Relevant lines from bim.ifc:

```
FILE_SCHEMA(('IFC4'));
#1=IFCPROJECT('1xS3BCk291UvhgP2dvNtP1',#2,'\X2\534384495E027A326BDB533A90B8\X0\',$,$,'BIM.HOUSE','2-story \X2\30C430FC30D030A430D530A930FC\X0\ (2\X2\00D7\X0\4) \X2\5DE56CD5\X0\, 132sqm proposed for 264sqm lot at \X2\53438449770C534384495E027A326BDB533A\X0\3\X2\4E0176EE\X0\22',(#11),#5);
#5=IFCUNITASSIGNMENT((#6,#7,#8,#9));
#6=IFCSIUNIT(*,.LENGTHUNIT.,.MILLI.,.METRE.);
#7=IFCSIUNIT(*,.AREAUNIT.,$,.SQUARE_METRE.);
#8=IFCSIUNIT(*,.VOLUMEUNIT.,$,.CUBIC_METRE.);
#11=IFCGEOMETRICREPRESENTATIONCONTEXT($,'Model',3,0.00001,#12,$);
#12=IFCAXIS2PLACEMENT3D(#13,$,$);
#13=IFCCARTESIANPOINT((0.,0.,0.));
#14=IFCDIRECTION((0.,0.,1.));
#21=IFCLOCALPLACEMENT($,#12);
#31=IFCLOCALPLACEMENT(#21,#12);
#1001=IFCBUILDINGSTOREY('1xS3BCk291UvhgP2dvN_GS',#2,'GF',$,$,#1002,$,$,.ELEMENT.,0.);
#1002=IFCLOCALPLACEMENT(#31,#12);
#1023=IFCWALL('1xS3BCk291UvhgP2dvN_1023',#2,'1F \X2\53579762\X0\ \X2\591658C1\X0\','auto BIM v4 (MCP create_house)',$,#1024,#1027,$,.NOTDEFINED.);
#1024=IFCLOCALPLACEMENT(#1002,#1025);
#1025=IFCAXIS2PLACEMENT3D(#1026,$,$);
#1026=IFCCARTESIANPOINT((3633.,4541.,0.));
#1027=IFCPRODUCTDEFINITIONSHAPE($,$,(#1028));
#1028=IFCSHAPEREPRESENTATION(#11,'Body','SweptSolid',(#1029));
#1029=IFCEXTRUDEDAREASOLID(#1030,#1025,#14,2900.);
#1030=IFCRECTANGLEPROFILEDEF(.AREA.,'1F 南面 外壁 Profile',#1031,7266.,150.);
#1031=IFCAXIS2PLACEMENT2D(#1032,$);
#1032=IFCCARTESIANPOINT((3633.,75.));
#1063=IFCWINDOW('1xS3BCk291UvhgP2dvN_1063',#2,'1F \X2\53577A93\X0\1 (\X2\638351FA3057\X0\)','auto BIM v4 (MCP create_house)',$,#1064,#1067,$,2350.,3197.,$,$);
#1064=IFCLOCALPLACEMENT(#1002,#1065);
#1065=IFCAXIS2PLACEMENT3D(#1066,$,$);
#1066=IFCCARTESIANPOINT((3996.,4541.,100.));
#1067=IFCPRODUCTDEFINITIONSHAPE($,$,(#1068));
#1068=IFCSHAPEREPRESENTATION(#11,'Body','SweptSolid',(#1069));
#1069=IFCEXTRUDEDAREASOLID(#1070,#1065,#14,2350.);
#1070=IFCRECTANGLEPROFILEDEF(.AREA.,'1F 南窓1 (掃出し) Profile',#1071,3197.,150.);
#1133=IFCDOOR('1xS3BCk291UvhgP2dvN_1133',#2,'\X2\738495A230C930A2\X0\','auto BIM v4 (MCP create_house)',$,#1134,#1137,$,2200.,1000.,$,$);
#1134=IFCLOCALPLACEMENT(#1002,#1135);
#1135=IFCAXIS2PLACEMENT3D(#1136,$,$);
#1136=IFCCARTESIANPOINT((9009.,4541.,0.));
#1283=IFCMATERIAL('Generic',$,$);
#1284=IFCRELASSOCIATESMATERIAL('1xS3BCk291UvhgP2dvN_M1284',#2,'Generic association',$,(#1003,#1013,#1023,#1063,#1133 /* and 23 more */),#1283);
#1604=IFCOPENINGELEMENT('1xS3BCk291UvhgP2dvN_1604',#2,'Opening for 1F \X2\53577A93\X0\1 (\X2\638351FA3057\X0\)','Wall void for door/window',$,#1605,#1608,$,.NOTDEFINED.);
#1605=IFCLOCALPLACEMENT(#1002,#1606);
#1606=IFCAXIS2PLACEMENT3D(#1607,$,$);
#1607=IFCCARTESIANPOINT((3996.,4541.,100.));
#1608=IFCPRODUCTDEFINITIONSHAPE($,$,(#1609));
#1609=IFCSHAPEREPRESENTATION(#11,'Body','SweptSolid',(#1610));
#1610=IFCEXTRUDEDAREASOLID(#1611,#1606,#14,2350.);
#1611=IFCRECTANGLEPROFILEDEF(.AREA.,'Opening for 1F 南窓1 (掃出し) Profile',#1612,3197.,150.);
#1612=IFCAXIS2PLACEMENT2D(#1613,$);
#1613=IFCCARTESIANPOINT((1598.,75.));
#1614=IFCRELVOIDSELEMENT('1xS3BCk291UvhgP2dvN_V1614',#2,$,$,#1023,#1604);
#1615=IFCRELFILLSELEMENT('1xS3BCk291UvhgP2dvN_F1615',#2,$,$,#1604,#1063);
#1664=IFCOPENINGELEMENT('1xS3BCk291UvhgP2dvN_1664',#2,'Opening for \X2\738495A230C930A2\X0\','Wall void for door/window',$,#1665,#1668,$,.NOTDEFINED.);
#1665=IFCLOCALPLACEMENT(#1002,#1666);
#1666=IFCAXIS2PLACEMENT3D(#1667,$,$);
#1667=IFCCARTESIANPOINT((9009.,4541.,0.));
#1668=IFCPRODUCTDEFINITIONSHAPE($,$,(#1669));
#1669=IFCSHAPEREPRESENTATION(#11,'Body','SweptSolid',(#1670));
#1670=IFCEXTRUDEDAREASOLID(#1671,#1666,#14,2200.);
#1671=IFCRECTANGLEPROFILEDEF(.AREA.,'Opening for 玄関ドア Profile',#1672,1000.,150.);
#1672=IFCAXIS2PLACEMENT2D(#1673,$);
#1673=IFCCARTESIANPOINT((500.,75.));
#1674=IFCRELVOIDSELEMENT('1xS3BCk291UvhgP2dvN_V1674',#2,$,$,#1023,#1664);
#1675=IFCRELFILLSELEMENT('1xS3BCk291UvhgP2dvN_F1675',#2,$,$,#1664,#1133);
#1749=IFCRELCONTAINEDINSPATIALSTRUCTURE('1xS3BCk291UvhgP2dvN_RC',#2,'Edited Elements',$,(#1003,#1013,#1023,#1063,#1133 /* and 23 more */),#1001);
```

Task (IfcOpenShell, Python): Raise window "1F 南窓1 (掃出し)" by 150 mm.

```python
import numpy as np
import ifcopenshell
import ifcopenshell.api.geometry
import ifcopenshell.util.placement
import ifcopenshell.util.unit

model = ifcopenshell.open("bim.ifc")
unit_scale = ifcopenshell.util.unit.calculate_unit_scale(model)

window = model.by_guid("1xS3BCk291UvhgP2dvN_1063")
opening = window.FillsVoids[0].RelatingOpeningElement
dz = 0.15 / unit_scale

shift = np.array([0.0, 0.0, dz])
# The window is not placed relative to its opening, so move both.
for product in (opening, window):
    matrix = ifcopenshell.util.placement.get_local_placement(product.ObjectPlacement)
    matrix[:3, 3] += shift
    ifcopenshell.api.geometry.edit_object_placement(model, product=product, matrix=matrix, is_si=False)

print(f"moved by {dz * unit_scale:+.3f} m")

model.write("bim-out.ifc")
```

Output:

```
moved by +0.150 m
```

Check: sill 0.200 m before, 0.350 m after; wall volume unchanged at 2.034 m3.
